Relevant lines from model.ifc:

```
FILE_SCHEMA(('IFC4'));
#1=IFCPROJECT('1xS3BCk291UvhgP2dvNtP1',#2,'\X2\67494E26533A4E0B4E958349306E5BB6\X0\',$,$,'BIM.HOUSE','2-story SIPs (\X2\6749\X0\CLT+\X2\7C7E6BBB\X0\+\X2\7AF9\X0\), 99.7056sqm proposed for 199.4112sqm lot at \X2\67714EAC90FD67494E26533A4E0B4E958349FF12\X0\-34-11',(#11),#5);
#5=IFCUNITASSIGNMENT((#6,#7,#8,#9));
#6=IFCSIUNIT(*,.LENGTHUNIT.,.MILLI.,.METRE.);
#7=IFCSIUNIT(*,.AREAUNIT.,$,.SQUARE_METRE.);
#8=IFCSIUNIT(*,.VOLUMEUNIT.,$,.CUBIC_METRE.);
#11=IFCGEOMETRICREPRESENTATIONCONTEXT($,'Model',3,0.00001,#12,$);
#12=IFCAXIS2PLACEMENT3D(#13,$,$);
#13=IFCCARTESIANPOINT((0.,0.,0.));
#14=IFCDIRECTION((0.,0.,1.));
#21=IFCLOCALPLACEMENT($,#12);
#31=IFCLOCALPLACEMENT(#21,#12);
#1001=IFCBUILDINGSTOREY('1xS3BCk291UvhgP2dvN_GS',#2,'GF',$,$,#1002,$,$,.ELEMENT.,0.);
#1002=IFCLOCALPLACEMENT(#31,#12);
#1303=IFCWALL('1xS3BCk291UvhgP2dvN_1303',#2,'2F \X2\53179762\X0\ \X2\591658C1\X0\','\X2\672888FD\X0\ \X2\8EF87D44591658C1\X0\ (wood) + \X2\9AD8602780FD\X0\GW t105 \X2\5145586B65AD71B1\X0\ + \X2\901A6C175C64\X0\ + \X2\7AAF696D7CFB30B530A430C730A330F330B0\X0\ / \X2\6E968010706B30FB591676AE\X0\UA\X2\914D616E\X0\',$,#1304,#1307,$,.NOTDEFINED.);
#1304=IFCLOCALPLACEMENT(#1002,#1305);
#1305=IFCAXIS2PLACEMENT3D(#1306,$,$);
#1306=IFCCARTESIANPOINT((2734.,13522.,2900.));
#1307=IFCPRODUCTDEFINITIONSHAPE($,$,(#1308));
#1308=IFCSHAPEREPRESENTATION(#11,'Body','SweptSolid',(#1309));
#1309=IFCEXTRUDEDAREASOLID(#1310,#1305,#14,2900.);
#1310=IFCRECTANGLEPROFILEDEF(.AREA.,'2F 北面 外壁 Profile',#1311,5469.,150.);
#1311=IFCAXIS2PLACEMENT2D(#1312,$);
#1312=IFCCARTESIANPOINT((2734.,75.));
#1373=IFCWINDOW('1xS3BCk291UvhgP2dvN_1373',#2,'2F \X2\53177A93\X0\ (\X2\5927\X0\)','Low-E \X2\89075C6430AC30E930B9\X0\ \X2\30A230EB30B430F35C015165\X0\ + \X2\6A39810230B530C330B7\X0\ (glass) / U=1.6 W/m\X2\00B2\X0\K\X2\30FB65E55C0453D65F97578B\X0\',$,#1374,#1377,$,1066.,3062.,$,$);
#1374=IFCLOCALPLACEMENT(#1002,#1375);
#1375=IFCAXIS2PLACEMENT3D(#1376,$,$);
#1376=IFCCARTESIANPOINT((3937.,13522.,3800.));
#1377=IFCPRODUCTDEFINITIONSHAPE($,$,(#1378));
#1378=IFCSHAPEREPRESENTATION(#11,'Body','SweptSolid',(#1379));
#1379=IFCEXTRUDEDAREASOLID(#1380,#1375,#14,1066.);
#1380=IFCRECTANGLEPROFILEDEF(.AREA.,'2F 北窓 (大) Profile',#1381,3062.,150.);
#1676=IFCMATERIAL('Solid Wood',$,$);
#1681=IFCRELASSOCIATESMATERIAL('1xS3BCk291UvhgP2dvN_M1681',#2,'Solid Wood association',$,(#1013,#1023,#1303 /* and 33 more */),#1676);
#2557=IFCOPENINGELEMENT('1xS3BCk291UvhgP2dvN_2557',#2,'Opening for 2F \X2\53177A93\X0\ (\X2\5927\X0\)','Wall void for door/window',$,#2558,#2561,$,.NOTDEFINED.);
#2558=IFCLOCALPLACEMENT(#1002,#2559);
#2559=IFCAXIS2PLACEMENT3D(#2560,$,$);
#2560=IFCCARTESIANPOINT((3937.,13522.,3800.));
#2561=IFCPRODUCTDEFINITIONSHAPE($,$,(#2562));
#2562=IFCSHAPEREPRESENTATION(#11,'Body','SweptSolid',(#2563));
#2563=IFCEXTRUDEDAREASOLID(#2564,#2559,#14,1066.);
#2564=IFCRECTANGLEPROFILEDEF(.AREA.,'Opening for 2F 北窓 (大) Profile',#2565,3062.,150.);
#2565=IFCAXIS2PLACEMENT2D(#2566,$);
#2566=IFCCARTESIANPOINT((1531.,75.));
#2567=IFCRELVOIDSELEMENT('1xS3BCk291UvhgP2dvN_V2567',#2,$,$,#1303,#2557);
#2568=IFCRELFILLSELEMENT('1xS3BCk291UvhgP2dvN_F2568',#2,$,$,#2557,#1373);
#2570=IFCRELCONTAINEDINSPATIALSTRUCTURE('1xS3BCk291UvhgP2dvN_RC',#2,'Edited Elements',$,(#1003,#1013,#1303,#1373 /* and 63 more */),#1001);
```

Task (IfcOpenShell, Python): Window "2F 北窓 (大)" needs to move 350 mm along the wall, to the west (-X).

```python
import ifcopenshell
import ifcopenshell.api.geometry
import ifcopenshell.util.placement

model = ifcopenshell.open("model.ifc")

window = model.by_guid("1xS3BCk291UvhgP2dvN_1373")
opening = window.FillsVoids[0].RelatingOpeningElement
wall = opening.VoidsElements[0].RelatingBuildingElement

wall_matrix = ifcopenshell.util.placement.get_local_placement(wall.ObjectPlacement)
shift = wall_matrix[:3, 0] * -350.0
before = ifcopenshell.util.placement.get_local_placement(window.ObjectPlacement)[:3, 3].copy()

# The window is not placed relative to its opening, so move both.
for product in (opening, window):
    matrix = ifcopenshell.util.placement.get_local_placement(product.ObjectPlacement)
    matrix[:3, 3] += shift
    ifcopenshell.api.geometry.edit_object_placement(model, product=product, matrix=matrix, is_si=False)

after = ifcopenshell.util.placement.get_local_placement(window.ObjectPlacement)[:3, 3]
print("window moved by", (after - before).round(3) + 0.0)

model.write("model_v2.ifc")
```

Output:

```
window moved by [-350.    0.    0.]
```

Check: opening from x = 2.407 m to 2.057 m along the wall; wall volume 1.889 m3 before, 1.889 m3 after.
